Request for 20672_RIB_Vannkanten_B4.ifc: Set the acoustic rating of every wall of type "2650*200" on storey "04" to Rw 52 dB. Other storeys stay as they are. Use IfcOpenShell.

First a look at what the model holds.

```python
import ifcopenshell
import ifcopenshell.util.element

model = ifcopenshell.open("20672_RIB_Vannkanten_B4.ifc")
print(model.schema)
storey = next(s for s in model.by_type("IfcBuildingStorey") if s.Name == "04")
walls = [e for e in ifcopenshell.util.element.get_decomposition(storey) if e.is_a("IfcWall")]
seen = {}
for e in walls:
    element_type = ifcopenshell.util.element.get_type(e)
    key = (element_type.Name if element_type != e and element_type else None, ifcopenshell.util.element.get_pset(e, "Pset_WallCommon", "AcousticRating"))
    seen[key] = seen.get(key, 0) + 1
for (name, value), count in sorted(seen.items(), key=str):
    print(count, "x", name, "|", value)
```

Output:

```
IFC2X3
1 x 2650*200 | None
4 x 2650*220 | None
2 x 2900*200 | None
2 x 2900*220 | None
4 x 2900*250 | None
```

```python
import ifcopenshell
import ifcopenshell.api.pset
import ifcopenshell.util.element

model = ifcopenshell.open("20672_RIB_Vannkanten_B4.ifc")

storey = next(s for s in model.by_type("IfcBuildingStorey") if s.Name == "04")
walls = [e for e in ifcopenshell.util.element.get_decomposition(storey) if e.is_a("IfcWall")]

count = 0
for e in walls:
    element_type = ifcopenshell.util.element.get_type(e)
    if element_type in (None, e) or element_type.Name != "2650*200":
        continue
    # add_pset returns the element's existing set when there is one.
    pset = ifcopenshell.api.pset.add_pset(model, product=e, name="Pset_WallCommon")
    ifcopenshell.api.pset.edit_pset(model, pset=pset, properties={"AcousticRating": "Rw 52 dB"})
    count += 1

print(count, "walls updated")

model.write("20672_RIB_Vannkanten_B4_v2.ifc")
```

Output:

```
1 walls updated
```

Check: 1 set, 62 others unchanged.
